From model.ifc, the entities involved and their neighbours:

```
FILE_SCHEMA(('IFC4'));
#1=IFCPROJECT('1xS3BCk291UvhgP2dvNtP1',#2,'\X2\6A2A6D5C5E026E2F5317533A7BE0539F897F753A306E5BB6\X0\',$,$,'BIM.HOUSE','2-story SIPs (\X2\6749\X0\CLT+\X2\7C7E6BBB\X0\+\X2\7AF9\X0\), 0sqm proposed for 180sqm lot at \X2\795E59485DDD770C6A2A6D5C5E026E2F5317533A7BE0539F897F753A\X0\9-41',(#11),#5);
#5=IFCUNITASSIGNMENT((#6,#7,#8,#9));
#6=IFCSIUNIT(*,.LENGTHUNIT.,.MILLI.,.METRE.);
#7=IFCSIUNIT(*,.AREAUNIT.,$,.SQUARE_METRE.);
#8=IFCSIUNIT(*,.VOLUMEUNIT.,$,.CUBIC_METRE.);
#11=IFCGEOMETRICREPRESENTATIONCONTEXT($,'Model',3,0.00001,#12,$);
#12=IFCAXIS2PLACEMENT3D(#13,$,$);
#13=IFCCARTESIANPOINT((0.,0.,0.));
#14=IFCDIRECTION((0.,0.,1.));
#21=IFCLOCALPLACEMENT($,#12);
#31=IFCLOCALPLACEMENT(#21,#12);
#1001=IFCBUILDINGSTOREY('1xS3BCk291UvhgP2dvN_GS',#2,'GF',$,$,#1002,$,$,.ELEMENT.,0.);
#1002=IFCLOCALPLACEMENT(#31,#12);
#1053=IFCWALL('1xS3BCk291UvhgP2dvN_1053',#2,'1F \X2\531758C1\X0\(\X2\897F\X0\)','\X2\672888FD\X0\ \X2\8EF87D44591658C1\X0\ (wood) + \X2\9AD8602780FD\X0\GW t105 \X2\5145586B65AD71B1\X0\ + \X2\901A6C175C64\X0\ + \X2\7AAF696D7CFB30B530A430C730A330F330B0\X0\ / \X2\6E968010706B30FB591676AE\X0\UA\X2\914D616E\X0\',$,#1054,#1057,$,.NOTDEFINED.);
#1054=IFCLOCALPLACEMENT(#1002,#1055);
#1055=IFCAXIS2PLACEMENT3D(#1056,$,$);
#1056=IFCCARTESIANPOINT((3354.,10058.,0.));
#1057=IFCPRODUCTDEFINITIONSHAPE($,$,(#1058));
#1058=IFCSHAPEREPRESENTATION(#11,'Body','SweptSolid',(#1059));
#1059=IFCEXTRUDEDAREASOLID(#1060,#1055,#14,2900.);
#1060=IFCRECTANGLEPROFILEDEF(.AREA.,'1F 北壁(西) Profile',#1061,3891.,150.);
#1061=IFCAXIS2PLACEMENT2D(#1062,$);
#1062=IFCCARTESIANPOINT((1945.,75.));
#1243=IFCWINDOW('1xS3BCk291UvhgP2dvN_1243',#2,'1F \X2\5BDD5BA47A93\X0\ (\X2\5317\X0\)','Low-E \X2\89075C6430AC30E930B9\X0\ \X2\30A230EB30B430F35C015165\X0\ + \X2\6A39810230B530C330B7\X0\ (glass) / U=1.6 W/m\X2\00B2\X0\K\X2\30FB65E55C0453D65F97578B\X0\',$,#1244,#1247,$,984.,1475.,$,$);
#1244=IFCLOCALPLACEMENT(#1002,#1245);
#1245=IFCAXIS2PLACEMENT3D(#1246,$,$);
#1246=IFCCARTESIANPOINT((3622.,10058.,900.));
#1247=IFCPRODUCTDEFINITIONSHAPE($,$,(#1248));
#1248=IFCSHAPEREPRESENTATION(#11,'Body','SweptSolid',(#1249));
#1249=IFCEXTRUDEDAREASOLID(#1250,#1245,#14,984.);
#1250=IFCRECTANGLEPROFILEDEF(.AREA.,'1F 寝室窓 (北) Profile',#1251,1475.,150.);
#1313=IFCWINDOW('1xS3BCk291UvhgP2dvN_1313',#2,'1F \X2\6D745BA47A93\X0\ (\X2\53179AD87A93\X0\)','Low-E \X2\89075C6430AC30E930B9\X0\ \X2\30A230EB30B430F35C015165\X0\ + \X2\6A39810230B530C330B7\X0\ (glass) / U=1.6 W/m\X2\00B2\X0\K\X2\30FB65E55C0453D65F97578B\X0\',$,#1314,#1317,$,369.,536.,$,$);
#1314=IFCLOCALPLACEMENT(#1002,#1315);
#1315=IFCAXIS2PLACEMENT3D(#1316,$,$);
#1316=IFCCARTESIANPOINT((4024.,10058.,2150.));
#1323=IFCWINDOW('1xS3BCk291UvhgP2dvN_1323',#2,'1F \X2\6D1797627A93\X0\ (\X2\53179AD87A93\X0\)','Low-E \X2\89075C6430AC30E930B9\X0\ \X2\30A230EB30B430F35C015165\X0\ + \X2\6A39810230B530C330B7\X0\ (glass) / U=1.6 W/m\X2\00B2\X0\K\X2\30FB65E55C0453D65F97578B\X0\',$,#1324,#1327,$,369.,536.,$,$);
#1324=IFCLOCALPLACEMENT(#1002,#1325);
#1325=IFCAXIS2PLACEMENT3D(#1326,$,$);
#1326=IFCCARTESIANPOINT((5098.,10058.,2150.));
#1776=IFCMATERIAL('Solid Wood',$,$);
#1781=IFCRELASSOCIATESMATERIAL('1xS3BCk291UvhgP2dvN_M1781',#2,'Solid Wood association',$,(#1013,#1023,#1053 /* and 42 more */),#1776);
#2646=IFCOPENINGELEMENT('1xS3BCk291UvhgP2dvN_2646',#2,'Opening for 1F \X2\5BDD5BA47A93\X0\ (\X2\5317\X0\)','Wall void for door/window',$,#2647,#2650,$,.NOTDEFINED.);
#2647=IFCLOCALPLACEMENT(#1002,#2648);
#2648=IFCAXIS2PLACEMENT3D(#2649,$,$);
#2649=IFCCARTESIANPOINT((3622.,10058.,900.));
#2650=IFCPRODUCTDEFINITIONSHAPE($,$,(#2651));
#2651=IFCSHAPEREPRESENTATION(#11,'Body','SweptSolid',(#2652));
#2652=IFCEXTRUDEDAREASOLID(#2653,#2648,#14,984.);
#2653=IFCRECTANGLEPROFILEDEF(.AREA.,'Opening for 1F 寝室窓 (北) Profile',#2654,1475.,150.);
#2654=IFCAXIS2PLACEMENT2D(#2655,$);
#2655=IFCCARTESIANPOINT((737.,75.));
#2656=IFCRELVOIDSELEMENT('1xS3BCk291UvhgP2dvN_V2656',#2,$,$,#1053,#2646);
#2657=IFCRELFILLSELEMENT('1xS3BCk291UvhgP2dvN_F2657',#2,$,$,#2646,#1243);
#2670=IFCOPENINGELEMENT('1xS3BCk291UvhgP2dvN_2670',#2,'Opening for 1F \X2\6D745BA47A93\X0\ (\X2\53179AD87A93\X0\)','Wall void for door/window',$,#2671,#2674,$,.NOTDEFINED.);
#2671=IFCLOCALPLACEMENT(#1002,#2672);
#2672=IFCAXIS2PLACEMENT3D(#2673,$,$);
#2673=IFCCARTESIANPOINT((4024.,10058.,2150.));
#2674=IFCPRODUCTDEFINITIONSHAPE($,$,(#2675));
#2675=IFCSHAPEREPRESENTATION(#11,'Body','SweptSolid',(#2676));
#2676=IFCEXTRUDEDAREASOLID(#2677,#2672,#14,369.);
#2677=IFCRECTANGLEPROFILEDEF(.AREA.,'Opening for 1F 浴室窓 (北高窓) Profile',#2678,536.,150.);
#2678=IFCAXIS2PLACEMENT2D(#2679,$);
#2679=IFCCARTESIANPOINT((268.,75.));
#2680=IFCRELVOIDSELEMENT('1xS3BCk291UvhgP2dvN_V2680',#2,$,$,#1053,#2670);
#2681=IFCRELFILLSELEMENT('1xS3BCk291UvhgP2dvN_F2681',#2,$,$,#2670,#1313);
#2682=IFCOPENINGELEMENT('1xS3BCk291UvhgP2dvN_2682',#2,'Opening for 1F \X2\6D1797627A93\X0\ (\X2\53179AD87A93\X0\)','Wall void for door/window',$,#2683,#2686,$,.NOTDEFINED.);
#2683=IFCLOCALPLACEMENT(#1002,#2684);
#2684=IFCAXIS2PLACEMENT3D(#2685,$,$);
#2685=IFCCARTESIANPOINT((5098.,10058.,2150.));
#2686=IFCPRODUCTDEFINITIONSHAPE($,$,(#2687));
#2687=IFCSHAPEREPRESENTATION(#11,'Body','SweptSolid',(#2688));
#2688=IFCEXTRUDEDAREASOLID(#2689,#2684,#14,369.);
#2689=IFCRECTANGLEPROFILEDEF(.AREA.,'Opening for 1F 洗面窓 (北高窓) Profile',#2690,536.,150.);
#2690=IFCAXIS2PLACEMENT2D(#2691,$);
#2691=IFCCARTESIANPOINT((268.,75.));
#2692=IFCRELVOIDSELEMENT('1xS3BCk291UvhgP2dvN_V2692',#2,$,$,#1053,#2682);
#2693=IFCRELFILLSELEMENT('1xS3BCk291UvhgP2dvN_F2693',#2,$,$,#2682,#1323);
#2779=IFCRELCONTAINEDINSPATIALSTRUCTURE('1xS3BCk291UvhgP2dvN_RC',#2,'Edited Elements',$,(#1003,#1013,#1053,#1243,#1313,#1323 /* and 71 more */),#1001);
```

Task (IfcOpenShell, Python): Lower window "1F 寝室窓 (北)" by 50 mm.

```python
import numpy as np
import ifcopenshell
import ifcopenshell.api.geometry
import ifcopenshell.util.placement
import ifcopenshell.util.unit

model = ifcopenshell.open("model.ifc")
unit_scale = ifcopenshell.util.unit.calculate_unit_scale(model)

window = model.by_guid("1xS3BCk291UvhgP2dvN_1243")
opening = window.FillsVoids[0].RelatingOpeningElement
dz = -50.0

shift = np.array([0.0, 0.0, dz])
# The window is not placed relative to its opening, so move both.
for product in (opening, window):
    matrix = ifcopenshell.util.placement.get_local_placement(product.ObjectPlacement)
    matrix[:3, 3] += shift
    ifcopenshell.api.geometry.edit_object_placement(model, product=product, matrix=matrix, is_si=False)

print(f"moved by {dz * unit_scale:+.3f} m")

model.write("model_edited.ifc")
```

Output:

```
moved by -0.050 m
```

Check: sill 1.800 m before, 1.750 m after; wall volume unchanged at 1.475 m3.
